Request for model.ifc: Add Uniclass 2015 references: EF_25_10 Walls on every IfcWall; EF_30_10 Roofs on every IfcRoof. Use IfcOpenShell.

First a look at what the model holds.

```python
import ifcopenshell

model = ifcopenshell.open("model.ifc")
print(model.schema)
print("classifications:", [c.Name for c in model.by_type("IfcClassification")])
for ifc_class in ("IfcDoor", "IfcRoof", "IfcStair", "IfcWall", "IfcWindow"):
    print(ifc_class, len(model.by_type(ifc_class)))
```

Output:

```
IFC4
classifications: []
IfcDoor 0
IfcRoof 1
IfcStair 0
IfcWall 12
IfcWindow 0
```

```python
import ifcopenshell
import ifcopenshell.api.classification

model = ifcopenshell.open("model.ifc")

system = ifcopenshell.api.classification.add_classification(model, classification="Uniclass 2015")

codes = {
    "IfcWall": ("EF_25_10", "Walls"),
    "IfcRoof": ("EF_30_10", "Roofs"),
}
for ifc_class, (code, name) in codes.items():
    products = model.by_type(ifc_class)
    ifcopenshell.api.classification.add_reference(
        model, products=products, classification=system, identification=code, name=name
    )
    print(code, len(products))

model.write("model_v2.ifc")
```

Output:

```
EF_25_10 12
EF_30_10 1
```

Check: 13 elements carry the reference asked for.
